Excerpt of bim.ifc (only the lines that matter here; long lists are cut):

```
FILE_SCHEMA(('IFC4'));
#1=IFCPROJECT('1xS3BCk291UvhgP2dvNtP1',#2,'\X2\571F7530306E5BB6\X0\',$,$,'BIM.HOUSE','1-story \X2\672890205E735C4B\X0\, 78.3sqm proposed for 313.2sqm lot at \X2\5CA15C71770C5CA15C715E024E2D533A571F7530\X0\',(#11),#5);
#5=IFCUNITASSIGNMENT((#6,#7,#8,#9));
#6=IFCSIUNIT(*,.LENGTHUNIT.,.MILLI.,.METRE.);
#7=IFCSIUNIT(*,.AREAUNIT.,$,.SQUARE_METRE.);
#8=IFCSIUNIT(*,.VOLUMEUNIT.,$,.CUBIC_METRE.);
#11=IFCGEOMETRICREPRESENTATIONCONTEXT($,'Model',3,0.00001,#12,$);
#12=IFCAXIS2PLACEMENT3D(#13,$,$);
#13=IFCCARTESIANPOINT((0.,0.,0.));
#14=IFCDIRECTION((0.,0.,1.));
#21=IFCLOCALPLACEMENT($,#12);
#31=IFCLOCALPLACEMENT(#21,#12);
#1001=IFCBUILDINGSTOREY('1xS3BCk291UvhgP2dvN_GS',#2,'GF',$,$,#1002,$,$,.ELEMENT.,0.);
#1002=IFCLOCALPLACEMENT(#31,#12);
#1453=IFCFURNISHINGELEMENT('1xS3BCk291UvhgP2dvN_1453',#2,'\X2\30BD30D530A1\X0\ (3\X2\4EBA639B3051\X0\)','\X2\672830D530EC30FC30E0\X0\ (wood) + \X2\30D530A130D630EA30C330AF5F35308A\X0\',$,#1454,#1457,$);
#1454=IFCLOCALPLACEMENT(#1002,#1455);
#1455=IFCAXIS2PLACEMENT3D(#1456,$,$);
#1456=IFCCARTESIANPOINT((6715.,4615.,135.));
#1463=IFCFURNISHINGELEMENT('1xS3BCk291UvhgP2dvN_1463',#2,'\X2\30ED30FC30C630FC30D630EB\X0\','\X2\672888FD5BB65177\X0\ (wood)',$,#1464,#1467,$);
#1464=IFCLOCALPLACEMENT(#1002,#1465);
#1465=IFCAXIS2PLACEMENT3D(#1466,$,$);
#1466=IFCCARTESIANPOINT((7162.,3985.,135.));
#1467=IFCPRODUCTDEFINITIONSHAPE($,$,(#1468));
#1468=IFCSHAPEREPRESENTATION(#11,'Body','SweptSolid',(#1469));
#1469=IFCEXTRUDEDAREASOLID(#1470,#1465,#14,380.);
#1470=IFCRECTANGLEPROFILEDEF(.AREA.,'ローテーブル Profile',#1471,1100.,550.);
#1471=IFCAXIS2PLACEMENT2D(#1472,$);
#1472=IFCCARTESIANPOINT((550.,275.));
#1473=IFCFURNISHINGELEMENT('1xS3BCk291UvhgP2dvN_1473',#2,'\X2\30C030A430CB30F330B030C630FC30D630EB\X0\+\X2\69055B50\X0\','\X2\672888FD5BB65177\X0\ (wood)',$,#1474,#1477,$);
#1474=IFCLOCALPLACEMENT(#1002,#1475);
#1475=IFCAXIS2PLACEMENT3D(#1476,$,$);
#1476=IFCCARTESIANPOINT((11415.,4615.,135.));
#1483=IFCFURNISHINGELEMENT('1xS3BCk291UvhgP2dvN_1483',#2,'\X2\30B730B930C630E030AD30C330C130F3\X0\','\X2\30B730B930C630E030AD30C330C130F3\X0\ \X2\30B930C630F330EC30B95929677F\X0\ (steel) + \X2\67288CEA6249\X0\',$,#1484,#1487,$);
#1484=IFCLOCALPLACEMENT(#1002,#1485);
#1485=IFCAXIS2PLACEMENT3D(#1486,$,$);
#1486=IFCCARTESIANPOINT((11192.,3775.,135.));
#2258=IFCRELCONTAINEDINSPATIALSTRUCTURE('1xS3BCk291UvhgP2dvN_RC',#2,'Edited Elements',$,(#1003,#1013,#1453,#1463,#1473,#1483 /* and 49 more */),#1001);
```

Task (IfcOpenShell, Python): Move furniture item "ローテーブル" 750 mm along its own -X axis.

```python
import ifcopenshell
import ifcopenshell.api.geometry
import ifcopenshell.util.placement

model = ifcopenshell.open("bim.ifc")

item = model.by_guid("1xS3BCk291UvhgP2dvN_1463")
matrix = ifcopenshell.util.placement.get_local_placement(item.ObjectPlacement)
matrix[:3, 3] -= matrix[:3, 0] * 750.0
ifcopenshell.api.geometry.edit_object_placement(model, product=item, matrix=matrix, is_si=False)

print(ifcopenshell.util.placement.get_local_placement(item.ObjectPlacement).round(3) + 0.0)

model.write("bim_v2.ifc")
```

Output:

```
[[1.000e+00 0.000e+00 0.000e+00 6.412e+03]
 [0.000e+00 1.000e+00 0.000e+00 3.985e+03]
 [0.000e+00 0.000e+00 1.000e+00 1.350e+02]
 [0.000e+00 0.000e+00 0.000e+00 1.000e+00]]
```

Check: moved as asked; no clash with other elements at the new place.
